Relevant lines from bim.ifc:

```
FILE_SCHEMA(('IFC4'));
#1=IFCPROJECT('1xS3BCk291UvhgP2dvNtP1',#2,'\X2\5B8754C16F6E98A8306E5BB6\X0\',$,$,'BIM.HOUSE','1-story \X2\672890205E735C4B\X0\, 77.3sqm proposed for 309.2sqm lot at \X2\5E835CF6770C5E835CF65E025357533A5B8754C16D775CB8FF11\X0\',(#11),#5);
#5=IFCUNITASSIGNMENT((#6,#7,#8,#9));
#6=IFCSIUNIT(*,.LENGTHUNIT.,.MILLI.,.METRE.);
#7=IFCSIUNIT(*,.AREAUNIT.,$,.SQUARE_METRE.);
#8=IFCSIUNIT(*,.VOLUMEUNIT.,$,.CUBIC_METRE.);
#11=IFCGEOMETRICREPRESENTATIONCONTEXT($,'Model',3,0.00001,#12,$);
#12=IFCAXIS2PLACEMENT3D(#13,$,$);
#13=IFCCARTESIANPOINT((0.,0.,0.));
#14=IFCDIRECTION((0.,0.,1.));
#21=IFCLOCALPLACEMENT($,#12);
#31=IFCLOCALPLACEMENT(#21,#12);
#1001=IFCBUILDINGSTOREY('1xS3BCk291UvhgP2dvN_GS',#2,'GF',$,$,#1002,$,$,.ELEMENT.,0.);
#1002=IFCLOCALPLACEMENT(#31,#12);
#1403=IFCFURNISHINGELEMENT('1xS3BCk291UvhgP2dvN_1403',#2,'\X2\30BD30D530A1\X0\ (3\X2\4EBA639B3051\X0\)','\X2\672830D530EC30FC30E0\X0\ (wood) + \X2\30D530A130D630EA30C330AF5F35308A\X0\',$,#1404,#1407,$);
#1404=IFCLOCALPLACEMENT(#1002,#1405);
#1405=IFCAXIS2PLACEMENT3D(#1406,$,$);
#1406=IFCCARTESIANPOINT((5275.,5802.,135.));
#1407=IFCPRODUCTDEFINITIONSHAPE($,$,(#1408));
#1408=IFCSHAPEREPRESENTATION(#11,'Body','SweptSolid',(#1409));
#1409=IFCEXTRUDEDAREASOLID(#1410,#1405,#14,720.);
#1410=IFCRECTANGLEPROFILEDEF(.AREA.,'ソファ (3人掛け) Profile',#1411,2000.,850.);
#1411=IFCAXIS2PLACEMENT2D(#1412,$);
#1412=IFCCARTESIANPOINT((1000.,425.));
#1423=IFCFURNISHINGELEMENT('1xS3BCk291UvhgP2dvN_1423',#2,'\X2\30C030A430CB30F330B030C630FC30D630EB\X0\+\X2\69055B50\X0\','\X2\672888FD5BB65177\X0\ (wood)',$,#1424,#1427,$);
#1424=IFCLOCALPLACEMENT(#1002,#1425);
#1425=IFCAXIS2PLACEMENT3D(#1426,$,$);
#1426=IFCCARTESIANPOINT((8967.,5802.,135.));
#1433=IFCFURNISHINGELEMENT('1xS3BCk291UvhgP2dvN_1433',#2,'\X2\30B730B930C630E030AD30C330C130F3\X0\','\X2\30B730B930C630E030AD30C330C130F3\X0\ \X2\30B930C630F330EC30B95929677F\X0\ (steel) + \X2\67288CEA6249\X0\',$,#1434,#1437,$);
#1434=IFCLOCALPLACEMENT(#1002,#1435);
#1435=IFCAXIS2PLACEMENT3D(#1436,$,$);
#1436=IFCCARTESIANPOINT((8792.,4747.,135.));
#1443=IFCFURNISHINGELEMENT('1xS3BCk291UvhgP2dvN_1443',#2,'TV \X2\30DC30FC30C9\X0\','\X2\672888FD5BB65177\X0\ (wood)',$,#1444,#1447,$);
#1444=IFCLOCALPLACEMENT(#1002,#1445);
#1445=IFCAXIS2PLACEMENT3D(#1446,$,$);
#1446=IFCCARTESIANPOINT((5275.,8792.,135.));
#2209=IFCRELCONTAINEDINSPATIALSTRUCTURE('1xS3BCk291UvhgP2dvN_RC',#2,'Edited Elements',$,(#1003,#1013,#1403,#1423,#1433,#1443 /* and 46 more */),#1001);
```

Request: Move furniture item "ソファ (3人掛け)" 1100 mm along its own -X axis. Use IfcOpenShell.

```python
import ifcopenshell
import ifcopenshell.api.geometry
import ifcopenshell.util.placement
import ifcopenshell.util.unit

model = ifcopenshell.open("bim.ifc")
unit_scale = ifcopenshell.util.unit.calculate_unit_scale(model)

item = model.by_id(1403)
matrix = ifcopenshell.util.placement.get_local_placement(item.ObjectPlacement)
matrix[:3, 3] -= matrix[:3, 0] * 1.1 / unit_scale
ifcopenshell.api.geometry.edit_object_placement(model, product=item, matrix=matrix, is_si=False)

print(ifcopenshell.util.placement.get_local_placement(item.ObjectPlacement).round(3) + 0.0)

model.write("bim-out.ifc")
```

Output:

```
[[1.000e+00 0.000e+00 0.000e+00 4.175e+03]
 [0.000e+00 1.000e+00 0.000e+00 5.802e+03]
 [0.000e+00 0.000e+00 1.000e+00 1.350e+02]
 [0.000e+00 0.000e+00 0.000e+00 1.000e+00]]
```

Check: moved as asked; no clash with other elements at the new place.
